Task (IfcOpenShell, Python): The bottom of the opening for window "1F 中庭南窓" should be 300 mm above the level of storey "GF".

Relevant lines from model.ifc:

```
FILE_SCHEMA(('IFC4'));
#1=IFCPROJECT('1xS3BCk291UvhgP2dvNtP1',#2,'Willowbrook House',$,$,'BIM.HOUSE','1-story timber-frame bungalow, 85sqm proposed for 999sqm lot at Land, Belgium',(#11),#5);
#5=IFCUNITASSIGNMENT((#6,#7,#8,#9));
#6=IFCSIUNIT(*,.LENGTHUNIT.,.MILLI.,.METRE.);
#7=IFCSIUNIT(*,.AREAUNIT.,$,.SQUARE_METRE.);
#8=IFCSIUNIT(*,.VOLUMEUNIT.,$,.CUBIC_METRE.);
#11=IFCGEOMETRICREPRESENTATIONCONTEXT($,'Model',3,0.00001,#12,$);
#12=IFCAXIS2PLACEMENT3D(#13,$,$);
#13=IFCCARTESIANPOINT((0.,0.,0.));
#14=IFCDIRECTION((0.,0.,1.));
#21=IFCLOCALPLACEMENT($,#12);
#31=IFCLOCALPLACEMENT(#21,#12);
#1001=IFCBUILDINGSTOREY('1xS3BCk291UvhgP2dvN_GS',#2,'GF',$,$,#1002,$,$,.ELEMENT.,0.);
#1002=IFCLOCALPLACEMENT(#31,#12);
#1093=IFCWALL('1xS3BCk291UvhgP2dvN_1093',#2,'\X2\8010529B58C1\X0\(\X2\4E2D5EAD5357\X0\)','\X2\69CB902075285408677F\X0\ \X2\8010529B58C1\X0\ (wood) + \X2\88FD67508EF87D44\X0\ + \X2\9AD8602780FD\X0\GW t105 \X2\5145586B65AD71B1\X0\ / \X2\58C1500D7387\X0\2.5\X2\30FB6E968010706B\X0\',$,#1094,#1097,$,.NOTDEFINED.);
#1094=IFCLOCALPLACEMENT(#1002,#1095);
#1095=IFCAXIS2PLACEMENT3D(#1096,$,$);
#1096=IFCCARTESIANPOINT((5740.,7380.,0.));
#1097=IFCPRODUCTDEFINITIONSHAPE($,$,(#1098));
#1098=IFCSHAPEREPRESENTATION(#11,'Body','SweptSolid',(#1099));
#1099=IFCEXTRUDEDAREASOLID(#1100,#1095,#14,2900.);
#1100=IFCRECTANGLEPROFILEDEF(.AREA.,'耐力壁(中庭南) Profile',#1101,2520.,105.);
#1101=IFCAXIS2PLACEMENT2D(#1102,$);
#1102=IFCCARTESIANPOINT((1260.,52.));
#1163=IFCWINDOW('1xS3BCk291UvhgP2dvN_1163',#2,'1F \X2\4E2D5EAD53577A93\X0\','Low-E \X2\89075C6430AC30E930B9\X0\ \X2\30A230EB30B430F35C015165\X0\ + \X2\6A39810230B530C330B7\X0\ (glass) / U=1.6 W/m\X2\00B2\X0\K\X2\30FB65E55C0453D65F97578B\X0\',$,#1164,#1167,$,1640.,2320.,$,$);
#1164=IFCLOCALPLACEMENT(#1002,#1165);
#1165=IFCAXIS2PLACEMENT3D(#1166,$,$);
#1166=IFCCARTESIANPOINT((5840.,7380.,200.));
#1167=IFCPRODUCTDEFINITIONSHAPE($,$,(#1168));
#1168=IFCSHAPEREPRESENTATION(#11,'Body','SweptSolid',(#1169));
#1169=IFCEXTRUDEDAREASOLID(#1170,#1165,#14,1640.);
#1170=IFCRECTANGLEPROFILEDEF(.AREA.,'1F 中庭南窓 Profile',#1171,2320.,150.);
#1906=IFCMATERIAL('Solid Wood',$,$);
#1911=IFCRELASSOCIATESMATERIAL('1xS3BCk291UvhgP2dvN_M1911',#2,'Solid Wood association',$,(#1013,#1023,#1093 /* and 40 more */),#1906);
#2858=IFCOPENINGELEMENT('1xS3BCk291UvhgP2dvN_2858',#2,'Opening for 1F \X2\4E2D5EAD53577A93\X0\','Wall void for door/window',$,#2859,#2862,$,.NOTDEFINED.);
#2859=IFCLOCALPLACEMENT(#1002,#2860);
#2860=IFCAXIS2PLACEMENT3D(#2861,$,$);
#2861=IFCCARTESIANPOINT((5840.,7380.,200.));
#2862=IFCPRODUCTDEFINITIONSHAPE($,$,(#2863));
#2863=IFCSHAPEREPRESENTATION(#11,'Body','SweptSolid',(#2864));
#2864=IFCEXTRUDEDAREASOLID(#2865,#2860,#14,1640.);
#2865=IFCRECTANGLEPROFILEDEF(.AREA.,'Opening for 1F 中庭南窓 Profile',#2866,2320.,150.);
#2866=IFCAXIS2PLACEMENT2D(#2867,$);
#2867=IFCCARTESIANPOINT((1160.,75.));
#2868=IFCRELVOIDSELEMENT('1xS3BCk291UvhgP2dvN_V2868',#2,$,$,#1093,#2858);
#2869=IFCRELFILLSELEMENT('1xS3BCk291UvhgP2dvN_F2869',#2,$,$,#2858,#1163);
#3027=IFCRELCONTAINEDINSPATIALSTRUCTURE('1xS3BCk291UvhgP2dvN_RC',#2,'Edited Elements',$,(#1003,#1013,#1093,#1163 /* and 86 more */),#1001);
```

```python
import numpy as np
import ifcopenshell
import ifcopenshell.api.geometry
import ifcopenshell.geom
import ifcopenshell.util.element
import ifcopenshell.util.placement
import ifcopenshell.util.shape
import ifcopenshell.util.unit

model = ifcopenshell.open("model.ifc")
unit_scale = ifcopenshell.util.unit.calculate_unit_scale(model)

window = model.by_id(1163)
opening = window.FillsVoids[0].RelatingOpeningElement
storey = ifcopenshell.util.element.get_container(window, ifc_class="IfcBuildingStorey")
level = ifcopenshell.util.placement.get_local_placement(storey.ObjectPlacement)[2, 3]

# The opening's origin need not be at the sill, so measure its lowest point.
shape = ifcopenshell.geom.create_shape(ifcopenshell.geom.settings(), opening)
bottom = ifcopenshell.util.shape.get_shape_bottom_elevation(shape, shape.geometry) / unit_scale
dz = level + 0.3 / unit_scale - bottom

shift = np.array([0.0, 0.0, dz])
# The window is not placed relative to its opening, so move both.
for product in (opening, window):
    matrix = ifcopenshell.util.placement.get_local_placement(product.ObjectPlacement)
    matrix[:3, 3] += shift
    ifcopenshell.api.geometry.edit_object_placement(model, product=product, matrix=matrix, is_si=False)

print(f"moved by {dz * unit_scale:+.3f} m")

model.write("model_edited.ifc")
```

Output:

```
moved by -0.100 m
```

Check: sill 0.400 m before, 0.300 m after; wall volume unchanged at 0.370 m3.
